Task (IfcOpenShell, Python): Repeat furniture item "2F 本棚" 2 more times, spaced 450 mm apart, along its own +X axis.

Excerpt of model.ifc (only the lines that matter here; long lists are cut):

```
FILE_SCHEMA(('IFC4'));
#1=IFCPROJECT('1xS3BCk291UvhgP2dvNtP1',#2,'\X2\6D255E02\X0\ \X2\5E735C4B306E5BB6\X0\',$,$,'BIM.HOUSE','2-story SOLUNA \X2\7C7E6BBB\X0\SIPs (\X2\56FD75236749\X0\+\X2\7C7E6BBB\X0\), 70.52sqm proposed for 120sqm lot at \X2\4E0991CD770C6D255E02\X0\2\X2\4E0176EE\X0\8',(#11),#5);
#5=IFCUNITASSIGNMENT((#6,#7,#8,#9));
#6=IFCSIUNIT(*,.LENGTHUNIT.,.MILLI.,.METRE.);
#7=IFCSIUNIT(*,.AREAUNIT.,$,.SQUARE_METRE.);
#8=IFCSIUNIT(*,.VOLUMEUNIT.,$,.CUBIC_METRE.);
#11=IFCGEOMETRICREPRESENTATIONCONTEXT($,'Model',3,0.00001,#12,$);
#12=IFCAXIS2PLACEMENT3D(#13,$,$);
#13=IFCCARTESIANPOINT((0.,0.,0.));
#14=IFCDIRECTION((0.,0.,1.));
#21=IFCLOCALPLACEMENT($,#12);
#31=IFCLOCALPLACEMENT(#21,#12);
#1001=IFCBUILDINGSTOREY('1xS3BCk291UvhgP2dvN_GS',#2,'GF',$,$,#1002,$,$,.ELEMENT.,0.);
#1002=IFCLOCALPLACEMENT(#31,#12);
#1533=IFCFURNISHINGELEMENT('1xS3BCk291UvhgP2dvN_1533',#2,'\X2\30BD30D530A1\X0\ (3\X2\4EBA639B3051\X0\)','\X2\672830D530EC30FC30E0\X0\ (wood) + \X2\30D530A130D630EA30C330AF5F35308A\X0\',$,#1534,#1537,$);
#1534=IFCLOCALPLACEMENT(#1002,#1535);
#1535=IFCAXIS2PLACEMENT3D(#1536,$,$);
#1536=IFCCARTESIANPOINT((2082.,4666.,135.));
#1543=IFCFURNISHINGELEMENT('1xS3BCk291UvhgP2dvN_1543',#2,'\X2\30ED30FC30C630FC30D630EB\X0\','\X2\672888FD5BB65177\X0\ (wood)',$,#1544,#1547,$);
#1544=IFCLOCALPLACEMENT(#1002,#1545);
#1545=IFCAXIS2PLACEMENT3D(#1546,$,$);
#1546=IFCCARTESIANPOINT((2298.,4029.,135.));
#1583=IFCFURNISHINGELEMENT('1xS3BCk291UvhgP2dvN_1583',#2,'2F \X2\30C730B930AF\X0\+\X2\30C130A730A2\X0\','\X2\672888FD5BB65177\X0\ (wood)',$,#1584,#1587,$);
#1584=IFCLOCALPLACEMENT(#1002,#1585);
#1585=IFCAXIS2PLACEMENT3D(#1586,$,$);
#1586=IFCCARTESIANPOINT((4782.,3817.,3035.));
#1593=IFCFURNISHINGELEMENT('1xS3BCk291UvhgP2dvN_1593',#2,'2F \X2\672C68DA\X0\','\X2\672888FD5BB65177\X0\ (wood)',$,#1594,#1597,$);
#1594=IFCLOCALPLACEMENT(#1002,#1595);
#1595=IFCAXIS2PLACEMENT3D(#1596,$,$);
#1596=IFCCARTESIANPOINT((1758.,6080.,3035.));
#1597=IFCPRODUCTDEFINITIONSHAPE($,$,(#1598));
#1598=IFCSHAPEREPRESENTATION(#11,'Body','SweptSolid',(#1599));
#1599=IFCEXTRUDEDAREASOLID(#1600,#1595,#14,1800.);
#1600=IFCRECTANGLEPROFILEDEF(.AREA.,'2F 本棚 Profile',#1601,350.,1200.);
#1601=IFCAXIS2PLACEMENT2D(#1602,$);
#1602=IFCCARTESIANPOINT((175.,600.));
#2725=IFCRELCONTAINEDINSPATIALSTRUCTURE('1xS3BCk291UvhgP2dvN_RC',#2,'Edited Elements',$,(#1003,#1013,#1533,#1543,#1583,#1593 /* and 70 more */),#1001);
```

```python
import ifcopenshell
import ifcopenshell.api.geometry
import ifcopenshell.api.root
import ifcopenshell.util.element
import ifcopenshell.util.placement

model = ifcopenshell.open("model.ifc")


def reuse_history(source, copy):
    """copy_class also copies each property set's owner history, people and application; keep the originals."""
    for rel in copy.IsDefinedBy:
        if rel.is_a("IfcRelDefinesByProperties") and (history := rel.RelatingPropertyDefinition.OwnerHistory):
            rel.RelatingPropertyDefinition.OwnerHistory = source.OwnerHistory
            ifcopenshell.util.element.remove_deep2(model, history)


source = model.by_guid("1xS3BCk291UvhgP2dvN_1593")
base = ifcopenshell.util.placement.get_local_placement(source.ObjectPlacement)
step = base[:3, 0] * 450.0

for i in range(1, 3):
    copy = ifcopenshell.api.root.copy_class(model, product=source)
    copy.Representation = ifcopenshell.util.element.copy_deep(
        model, source.Representation, exclude=["IfcGeometricRepresentationContext", "IfcRepresentationMap"]
    )
    reuse_history(source, copy)
    matrix = base.copy()
    matrix[:3, 3] += i * step
    print("added at", matrix[:3, 3].round(3) + 0.0)
    ifcopenshell.api.geometry.edit_object_placement(model, product=copy, matrix=matrix, is_si=False)

model.write("model_v2.ifc")
```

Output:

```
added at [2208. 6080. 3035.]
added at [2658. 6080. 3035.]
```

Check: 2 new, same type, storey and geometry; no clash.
